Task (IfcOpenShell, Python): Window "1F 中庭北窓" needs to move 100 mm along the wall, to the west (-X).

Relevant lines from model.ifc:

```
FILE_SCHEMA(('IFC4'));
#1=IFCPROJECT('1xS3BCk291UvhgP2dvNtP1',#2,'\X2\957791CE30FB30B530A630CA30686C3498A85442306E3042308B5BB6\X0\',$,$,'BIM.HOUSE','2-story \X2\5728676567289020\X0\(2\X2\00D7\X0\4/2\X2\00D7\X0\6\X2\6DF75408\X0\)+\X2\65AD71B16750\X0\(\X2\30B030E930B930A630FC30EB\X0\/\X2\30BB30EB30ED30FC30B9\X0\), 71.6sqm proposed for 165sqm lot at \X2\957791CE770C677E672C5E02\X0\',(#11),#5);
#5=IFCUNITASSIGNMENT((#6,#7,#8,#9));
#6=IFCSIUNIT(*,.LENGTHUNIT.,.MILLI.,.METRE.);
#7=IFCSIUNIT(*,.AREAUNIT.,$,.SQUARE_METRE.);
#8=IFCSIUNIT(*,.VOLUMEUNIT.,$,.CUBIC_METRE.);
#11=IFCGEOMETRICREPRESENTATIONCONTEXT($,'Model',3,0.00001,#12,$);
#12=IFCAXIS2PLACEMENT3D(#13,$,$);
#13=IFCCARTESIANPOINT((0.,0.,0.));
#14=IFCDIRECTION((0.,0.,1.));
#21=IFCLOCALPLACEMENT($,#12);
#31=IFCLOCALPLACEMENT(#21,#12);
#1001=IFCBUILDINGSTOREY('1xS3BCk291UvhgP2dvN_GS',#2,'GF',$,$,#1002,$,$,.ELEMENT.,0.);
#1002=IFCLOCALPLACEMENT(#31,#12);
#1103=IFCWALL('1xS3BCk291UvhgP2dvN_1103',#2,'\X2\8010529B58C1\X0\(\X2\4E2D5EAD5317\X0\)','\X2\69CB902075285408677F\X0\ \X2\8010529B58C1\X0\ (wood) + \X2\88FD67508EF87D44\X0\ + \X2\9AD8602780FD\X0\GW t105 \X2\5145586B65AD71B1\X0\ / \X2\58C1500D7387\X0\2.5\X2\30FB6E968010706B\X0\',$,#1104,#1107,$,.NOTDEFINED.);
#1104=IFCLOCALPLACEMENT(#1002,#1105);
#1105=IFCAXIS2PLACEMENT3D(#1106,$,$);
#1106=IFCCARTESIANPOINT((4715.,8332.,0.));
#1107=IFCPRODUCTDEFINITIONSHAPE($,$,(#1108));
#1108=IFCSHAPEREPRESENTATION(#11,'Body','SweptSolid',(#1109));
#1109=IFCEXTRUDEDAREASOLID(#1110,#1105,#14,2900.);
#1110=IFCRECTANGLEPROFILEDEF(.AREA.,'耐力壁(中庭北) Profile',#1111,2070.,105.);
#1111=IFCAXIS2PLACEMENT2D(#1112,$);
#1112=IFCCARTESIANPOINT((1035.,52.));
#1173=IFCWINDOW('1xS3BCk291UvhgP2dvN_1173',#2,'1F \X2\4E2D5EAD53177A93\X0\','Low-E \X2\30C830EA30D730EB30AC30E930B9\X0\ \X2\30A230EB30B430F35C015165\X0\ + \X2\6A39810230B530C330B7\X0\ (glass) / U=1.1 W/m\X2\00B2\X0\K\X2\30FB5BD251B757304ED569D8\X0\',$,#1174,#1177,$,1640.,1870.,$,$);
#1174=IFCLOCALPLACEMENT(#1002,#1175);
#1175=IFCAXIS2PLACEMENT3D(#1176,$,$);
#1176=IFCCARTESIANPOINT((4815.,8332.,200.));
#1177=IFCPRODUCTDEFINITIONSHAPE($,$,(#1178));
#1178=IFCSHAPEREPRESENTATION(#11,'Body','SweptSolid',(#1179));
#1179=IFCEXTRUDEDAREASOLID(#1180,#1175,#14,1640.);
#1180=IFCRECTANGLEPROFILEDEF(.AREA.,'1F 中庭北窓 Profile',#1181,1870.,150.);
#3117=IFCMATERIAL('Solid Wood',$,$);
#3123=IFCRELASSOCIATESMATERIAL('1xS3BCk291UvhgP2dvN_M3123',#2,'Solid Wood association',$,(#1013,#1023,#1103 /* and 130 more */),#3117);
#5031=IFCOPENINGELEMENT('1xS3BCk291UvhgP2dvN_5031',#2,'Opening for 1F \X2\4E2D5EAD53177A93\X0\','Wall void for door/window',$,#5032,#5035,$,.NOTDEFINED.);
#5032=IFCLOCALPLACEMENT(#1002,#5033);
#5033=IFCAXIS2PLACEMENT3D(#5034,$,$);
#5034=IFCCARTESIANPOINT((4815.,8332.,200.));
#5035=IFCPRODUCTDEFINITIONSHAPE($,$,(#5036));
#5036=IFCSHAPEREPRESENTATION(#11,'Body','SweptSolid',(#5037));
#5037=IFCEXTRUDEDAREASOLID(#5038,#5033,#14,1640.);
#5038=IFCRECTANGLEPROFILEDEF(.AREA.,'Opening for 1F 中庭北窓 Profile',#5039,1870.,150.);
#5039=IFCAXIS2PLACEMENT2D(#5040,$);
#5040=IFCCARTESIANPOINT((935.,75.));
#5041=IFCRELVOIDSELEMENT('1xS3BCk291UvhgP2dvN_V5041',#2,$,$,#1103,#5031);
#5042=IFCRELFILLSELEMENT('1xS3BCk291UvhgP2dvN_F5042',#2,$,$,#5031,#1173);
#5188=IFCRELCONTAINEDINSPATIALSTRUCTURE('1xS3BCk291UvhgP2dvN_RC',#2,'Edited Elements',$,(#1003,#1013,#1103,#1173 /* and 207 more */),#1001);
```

```python
import ifcopenshell
import ifcopenshell.api.geometry
import ifcopenshell.util.placement
import ifcopenshell.util.unit

model = ifcopenshell.open("model.ifc")
unit_scale = ifcopenshell.util.unit.calculate_unit_scale(model)

window = model.by_guid("1xS3BCk291UvhgP2dvN_1173")
opening = window.FillsVoids[0].RelatingOpeningElement
wall = opening.VoidsElements[0].RelatingBuildingElement

wall_matrix = ifcopenshell.util.placement.get_local_placement(wall.ObjectPlacement)
shift = wall_matrix[:3, 0] * -0.1 / unit_scale
before = ifcopenshell.util.placement.get_local_placement(window.ObjectPlacement)[:3, 3].copy()

# The window is not placed relative to its opening, so move both.
for product in (opening, window):
    matrix = ifcopenshell.util.placement.get_local_placement(product.ObjectPlacement)
    matrix[:3, 3] += shift
    ifcopenshell.api.geometry.edit_object_placement(model, product=product, matrix=matrix, is_si=False)

after = ifcopenshell.util.placement.get_local_placement(window.ObjectPlacement)[:3, 3]
print("window moved by", (after - before).round(3) + 0.0)

model.write("model-out.ifc")
```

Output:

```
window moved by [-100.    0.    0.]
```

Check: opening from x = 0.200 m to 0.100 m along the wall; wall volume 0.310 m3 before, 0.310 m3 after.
